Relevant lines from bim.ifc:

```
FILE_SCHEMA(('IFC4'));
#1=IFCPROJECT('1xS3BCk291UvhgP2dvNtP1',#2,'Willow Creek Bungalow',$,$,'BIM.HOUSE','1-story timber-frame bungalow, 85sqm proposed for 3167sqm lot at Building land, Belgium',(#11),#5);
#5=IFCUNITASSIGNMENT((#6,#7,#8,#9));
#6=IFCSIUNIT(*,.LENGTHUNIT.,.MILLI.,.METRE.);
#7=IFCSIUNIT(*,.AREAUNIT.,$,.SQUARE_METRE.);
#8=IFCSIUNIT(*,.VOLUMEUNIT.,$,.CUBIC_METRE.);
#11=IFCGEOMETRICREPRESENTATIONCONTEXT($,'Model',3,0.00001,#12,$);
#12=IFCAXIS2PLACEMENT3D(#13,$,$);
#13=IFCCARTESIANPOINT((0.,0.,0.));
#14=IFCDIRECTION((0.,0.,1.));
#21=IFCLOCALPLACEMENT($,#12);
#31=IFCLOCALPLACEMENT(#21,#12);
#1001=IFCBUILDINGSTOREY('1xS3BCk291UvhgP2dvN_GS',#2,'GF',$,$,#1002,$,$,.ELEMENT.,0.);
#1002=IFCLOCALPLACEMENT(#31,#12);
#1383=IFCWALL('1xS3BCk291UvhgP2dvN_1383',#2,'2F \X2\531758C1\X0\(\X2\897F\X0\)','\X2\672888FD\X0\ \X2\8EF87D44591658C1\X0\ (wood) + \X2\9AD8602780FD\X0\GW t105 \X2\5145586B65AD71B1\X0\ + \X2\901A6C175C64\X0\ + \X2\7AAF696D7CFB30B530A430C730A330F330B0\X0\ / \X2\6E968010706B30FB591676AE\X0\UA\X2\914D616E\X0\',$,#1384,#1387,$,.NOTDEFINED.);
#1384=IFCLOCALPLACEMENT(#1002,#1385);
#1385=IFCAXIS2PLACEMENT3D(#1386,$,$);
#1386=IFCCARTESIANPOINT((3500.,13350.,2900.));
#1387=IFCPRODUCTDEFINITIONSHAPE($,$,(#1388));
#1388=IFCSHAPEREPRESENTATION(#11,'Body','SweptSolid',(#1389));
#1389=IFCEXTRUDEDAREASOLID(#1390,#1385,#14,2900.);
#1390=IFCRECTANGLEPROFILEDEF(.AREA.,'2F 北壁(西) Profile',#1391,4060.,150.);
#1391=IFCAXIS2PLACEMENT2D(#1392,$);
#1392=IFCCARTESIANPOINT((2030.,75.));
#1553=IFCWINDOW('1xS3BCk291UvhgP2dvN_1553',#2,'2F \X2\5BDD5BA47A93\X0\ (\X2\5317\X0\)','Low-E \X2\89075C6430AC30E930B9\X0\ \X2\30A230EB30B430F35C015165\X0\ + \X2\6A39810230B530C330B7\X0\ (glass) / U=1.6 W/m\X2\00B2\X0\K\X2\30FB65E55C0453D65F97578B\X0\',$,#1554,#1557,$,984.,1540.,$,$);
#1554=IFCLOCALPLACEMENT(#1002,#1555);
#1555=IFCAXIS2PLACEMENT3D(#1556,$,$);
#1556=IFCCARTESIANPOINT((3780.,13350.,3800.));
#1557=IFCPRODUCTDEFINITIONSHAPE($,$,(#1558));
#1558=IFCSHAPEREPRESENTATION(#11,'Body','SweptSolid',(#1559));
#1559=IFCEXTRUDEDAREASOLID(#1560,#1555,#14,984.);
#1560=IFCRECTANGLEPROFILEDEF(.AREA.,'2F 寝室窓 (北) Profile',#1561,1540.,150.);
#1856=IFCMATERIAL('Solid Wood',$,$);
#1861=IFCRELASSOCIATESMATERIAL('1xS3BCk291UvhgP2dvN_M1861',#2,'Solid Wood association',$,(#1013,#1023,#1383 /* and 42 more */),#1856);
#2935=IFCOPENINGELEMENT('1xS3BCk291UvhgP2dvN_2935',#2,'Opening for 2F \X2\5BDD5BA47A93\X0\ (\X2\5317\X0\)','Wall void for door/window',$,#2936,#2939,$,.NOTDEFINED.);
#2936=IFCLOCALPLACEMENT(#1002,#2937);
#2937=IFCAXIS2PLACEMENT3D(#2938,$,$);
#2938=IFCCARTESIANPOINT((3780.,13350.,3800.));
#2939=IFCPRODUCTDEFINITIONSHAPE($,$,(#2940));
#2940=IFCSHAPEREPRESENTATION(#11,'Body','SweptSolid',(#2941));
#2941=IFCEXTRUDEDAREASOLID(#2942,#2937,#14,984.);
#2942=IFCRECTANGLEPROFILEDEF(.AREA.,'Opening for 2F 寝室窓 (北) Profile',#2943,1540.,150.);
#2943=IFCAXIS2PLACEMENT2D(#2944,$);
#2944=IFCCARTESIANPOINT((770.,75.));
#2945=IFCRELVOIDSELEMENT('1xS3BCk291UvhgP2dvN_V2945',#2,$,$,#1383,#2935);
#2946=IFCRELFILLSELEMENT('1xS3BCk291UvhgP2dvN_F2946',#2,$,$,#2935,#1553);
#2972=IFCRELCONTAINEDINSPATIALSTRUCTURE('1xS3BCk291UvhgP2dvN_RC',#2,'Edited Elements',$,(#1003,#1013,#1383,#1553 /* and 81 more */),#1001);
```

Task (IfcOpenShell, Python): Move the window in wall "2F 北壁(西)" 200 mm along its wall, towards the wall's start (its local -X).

```python
import ifcopenshell
import ifcopenshell.api.geometry
import ifcopenshell.util.placement

model = ifcopenshell.open("bim.ifc")

window = model.by_guid("1xS3BCk291UvhgP2dvN_1553")
opening = window.FillsVoids[0].RelatingOpeningElement
wall = opening.VoidsElements[0].RelatingBuildingElement

wall_matrix = ifcopenshell.util.placement.get_local_placement(wall.ObjectPlacement)
shift = wall_matrix[:3, 0] * -200.0
before = ifcopenshell.util.placement.get_local_placement(window.ObjectPlacement)[:3, 3].copy()

# The window is not placed relative to its opening, so move both.
for product in (opening, window):
    matrix = ifcopenshell.util.placement.get_local_placement(product.ObjectPlacement)
    matrix[:3, 3] += shift
    ifcopenshell.api.geometry.edit_object_placement(model, product=product, matrix=matrix, is_si=False)

after = ifcopenshell.util.placement.get_local_placement(window.ObjectPlacement)[:3, 3]
print("window moved by", (after - before).round(3) + 0.0)

model.write("bim_updated.ifc")
```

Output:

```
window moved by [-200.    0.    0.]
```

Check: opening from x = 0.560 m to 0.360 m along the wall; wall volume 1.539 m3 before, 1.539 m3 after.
